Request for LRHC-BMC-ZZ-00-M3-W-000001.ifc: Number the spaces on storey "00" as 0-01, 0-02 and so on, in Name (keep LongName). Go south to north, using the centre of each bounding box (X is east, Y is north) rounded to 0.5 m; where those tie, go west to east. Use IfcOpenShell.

First a look at what the model holds.

```python
import ifcopenshell
import ifcopenshell.util.element
import ifcopenshell.util.placement

model = ifcopenshell.open("LRHC-BMC-ZZ-00-M3-W-000001.ifc")
print(model.schema)
storey = next(s for s in model.by_type("IfcBuildingStorey") if s.Name == "00")
spaces = [e for e in ifcopenshell.util.element.get_decomposition(storey) if e.is_a("IfcSpace")]
for e in sorted(spaces, key=lambda e: e.id()):
    origin = ifcopenshell.util.placement.get_local_placement(e.ObjectPlacement)[:3, 3]
    print(e.id(), e.Name, e.LongName, origin.round(2) + 0.0, sep=" | ")
```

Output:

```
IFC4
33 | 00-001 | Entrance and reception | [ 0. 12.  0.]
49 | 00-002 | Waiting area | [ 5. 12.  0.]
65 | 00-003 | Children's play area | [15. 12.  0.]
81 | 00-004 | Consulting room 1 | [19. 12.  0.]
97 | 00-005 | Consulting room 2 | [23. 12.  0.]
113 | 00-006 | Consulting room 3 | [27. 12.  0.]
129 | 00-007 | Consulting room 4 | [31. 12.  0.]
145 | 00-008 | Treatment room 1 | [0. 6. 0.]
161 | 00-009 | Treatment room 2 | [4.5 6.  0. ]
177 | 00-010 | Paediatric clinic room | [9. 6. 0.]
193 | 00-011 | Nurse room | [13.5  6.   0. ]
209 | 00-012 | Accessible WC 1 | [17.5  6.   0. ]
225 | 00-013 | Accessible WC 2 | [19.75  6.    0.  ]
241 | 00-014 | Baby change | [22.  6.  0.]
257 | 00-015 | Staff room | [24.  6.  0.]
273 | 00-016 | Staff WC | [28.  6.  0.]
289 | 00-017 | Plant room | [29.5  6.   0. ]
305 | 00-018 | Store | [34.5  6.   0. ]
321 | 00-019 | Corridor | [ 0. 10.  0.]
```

```python
import ifcopenshell
import ifcopenshell.geom
import ifcopenshell.util.element
import ifcopenshell.util.shape

model = ifcopenshell.open("LRHC-BMC-ZZ-00-M3-W-000001.ifc")
settings = ifcopenshell.geom.settings()
settings.set("use-world-coords", True)


def centre(element):
    shape = ifcopenshell.geom.create_shape(settings, element)
    return ifcopenshell.util.shape.get_bbox_centroid(shape.geometry)


storey = next(s for s in model.by_type("IfcBuildingStorey") if s.Name == "00")
spaces = [e for e in ifcopenshell.util.element.get_decomposition(storey) if e.is_a("IfcSpace")]

# Insertion points can sit at a corner or the storey origin, so sort by the geometry (in metres).
centres = {e: centre(e) for e in spaces}
spaces.sort(key=lambda e: (round(centres[e][1] / 0.5), centres[e][0]))

for i, e in enumerate(spaces, start=1):
    number = f"0-{i:02d}"
    e.Name = number
    print(e.id(), number)

model.write("LRHC-BMC-ZZ-00-M3-W-000001_v2.ifc")
```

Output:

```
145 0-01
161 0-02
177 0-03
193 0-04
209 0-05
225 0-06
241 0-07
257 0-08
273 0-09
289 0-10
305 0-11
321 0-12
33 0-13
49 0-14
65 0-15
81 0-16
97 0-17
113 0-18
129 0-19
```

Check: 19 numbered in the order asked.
